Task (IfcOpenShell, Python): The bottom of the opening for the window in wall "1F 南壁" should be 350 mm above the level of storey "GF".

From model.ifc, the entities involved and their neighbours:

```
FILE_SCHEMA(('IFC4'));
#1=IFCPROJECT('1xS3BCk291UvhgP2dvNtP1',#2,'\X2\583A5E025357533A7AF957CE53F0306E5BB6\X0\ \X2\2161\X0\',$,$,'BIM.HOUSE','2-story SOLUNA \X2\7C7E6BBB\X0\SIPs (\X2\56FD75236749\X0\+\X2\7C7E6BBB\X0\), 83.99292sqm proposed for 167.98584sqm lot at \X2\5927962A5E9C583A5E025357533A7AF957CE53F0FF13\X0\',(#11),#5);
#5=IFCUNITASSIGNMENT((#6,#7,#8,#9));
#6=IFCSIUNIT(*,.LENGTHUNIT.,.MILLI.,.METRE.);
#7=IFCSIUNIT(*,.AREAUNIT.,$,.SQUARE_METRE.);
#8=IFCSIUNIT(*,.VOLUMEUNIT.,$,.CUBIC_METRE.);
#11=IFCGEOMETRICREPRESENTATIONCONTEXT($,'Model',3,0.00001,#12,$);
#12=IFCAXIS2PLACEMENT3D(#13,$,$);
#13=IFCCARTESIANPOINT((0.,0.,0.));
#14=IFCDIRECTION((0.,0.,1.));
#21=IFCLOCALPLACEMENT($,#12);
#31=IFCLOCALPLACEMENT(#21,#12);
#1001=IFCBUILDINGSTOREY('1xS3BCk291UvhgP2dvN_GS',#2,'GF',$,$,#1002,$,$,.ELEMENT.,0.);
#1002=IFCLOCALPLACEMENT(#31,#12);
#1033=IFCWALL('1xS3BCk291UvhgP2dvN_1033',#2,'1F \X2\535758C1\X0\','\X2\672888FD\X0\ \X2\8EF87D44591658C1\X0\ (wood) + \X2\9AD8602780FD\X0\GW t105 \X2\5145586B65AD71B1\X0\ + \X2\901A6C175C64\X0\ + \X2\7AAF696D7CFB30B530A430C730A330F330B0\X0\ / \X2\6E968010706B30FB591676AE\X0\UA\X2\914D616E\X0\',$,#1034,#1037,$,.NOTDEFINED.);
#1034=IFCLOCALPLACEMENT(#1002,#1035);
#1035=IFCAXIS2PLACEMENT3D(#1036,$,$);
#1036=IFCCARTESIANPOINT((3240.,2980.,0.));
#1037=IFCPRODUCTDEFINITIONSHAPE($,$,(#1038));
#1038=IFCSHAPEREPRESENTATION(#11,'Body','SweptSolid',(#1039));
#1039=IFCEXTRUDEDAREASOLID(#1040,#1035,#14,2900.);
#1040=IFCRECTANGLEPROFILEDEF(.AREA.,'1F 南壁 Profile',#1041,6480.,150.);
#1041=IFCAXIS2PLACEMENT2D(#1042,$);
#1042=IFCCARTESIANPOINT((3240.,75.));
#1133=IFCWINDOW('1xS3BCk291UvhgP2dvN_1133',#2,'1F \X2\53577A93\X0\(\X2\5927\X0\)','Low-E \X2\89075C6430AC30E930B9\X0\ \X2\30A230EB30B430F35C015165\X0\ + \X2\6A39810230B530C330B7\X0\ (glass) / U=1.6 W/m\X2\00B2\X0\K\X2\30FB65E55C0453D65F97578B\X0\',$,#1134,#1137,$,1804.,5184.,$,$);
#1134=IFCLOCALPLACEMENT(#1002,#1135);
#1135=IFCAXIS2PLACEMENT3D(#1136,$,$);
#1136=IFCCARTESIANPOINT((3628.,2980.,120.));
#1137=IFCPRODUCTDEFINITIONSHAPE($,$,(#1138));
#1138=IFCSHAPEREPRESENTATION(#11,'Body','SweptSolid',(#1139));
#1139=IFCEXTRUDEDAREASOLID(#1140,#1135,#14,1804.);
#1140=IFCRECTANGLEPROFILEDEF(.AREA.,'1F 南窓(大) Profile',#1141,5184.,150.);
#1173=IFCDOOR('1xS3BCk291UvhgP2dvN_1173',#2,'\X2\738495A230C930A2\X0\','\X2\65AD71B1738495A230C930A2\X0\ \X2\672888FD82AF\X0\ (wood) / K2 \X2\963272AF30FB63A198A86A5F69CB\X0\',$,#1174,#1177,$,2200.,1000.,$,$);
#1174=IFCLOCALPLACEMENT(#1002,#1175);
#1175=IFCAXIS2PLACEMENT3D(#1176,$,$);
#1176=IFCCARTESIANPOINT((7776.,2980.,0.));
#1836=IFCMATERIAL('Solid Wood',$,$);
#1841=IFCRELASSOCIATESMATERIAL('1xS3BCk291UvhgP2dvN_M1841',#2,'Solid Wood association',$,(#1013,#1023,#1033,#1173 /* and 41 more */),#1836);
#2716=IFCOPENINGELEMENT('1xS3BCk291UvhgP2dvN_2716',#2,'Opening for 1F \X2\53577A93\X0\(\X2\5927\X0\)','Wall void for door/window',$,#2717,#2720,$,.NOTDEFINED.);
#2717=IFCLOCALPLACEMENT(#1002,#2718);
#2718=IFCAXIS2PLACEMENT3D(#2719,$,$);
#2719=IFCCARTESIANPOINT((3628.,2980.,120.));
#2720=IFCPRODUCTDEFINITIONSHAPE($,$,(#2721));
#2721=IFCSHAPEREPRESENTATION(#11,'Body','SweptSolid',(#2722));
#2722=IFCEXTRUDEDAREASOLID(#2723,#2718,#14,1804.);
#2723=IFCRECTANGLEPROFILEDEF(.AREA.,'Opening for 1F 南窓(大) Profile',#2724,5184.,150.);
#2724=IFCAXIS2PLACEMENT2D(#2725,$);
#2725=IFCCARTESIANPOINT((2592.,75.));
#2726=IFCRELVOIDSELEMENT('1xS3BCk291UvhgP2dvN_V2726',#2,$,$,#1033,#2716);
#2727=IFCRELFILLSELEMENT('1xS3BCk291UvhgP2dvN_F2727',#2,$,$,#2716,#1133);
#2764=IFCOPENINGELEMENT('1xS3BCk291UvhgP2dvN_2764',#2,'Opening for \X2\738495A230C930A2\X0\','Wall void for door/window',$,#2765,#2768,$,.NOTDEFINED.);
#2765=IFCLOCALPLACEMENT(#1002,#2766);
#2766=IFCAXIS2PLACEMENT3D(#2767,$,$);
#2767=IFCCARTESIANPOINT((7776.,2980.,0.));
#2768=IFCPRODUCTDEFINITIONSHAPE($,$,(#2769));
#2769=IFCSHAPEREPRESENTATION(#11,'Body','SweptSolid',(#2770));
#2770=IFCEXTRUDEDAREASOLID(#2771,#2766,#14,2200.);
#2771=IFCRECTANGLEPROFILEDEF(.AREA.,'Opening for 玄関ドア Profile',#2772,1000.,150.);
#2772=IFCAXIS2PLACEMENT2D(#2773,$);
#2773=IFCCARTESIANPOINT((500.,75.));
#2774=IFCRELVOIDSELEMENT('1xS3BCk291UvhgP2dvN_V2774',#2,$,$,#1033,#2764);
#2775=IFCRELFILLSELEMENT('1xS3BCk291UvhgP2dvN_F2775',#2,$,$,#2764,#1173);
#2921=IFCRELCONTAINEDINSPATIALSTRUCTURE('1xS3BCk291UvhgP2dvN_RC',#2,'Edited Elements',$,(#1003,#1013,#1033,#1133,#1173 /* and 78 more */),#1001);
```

```python
import numpy as np
import ifcopenshell
import ifcopenshell.api.geometry
import ifcopenshell.geom
import ifcopenshell.util.element
import ifcopenshell.util.placement
import ifcopenshell.util.shape
import ifcopenshell.util.unit

model = ifcopenshell.open("model.ifc")
unit_scale = ifcopenshell.util.unit.calculate_unit_scale(model)

window = model.by_guid("1xS3BCk291UvhgP2dvN_1133")
opening = window.FillsVoids[0].RelatingOpeningElement
storey = ifcopenshell.util.element.get_container(window, ifc_class="IfcBuildingStorey")
level = ifcopenshell.util.placement.get_local_placement(storey.ObjectPlacement)[2, 3]

# The opening's origin need not be at the sill, so measure its lowest point.
shape = ifcopenshell.geom.create_shape(ifcopenshell.geom.settings(), opening)
bottom = ifcopenshell.util.shape.get_shape_bottom_elevation(shape, shape.geometry) / unit_scale
dz = level + 0.35 / unit_scale - bottom

shift = np.array([0.0, 0.0, dz])
# The window is not placed relative to its opening, so move both.
for product in (opening, window):
    matrix = ifcopenshell.util.placement.get_local_placement(product.ObjectPlacement)
    matrix[:3, 3] += shift
    ifcopenshell.api.geometry.edit_object_placement(model, product=product, matrix=matrix, is_si=False)

print(f"moved by {dz * unit_scale:+.3f} m")

model.write("model_updated.ifc")
```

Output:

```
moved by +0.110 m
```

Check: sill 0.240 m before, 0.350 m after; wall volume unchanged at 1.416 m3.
